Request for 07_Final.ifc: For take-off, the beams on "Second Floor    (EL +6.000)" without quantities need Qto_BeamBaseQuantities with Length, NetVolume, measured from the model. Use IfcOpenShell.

First a look at what the model holds.

```python
import ifcopenshell
import ifcopenshell.util.element
import ifcopenshell.util.unit

model = ifcopenshell.open("07_Final.ifc")
print(model.schema)
for unit_type in ("LENGTHUNIT", "AREAUNIT", "VOLUMEUNIT"):
    print(unit_type, ifcopenshell.util.unit.calculate_unit_scale(model, unit_type))
storey = next(s for s in model.by_type("IfcBuildingStorey") if s.Name == "Second Floor    (EL +6.000)")
beams = [e for e in ifcopenshell.util.element.get_decomposition(storey) if e.is_a("IfcBeam")]
for e in sorted(beams, key=lambda e: e.id()):
    print(e.id(), e.is_a(), e.Name, list(ifcopenshell.util.element.get_psets(e, qtos_only=True)), sep=" | ")
```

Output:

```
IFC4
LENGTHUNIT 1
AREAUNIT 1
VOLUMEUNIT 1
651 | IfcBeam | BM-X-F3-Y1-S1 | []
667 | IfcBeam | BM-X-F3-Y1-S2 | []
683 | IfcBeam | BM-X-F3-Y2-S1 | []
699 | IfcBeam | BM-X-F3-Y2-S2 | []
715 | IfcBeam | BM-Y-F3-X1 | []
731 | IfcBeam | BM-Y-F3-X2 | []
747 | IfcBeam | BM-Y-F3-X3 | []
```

```python
import ifcopenshell
import ifcopenshell.api.pset
import ifcopenshell.geom
import ifcopenshell.util.element
import ifcopenshell.util.shape
import ifcopenshell.util.unit

model = ifcopenshell.open("07_Final.ifc")
unit_scale = ifcopenshell.util.unit.calculate_unit_scale(model)
volume_scale = ifcopenshell.util.unit.calculate_unit_scale(model, "VOLUMEUNIT")
settings = ifcopenshell.geom.settings()

storey = next(s for s in model.by_type("IfcBuildingStorey") if s.Name == "Second Floor    (EL +6.000)")
beams = [e for e in ifcopenshell.util.element.get_decomposition(storey) if e.is_a("IfcBeam")]

for e in sorted(beams, key=lambda e: e.id()):
    if ifcopenshell.util.element.get_psets(e, qtos_only=True, should_inherit=False):
        continue
    # Geometry comes back in metres, in the element's own axes.
    shape = ifcopenshell.geom.create_shape(settings, e)
    values = {
        "Length": ifcopenshell.util.shape.get_max_xyz(shape.geometry) / unit_scale,
        "NetVolume": ifcopenshell.util.shape.get_volume(shape.geometry) / volume_scale,
    }
    qto = ifcopenshell.api.pset.add_qto(model, product=e, name="Qto_BeamBaseQuantities")
    ifcopenshell.api.pset.edit_qto(model, qto=qto, properties=values)
    print(e.id(), {k: round(v, 3) for k, v in values.items()})

model.write("07_Final_updated.ifc")
```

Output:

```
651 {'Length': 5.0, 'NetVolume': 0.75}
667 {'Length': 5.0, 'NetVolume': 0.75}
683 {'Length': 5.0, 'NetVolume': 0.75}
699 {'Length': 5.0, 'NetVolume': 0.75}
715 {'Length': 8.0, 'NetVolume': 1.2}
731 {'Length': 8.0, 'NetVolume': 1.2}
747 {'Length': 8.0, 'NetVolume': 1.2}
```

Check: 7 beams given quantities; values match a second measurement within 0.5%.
